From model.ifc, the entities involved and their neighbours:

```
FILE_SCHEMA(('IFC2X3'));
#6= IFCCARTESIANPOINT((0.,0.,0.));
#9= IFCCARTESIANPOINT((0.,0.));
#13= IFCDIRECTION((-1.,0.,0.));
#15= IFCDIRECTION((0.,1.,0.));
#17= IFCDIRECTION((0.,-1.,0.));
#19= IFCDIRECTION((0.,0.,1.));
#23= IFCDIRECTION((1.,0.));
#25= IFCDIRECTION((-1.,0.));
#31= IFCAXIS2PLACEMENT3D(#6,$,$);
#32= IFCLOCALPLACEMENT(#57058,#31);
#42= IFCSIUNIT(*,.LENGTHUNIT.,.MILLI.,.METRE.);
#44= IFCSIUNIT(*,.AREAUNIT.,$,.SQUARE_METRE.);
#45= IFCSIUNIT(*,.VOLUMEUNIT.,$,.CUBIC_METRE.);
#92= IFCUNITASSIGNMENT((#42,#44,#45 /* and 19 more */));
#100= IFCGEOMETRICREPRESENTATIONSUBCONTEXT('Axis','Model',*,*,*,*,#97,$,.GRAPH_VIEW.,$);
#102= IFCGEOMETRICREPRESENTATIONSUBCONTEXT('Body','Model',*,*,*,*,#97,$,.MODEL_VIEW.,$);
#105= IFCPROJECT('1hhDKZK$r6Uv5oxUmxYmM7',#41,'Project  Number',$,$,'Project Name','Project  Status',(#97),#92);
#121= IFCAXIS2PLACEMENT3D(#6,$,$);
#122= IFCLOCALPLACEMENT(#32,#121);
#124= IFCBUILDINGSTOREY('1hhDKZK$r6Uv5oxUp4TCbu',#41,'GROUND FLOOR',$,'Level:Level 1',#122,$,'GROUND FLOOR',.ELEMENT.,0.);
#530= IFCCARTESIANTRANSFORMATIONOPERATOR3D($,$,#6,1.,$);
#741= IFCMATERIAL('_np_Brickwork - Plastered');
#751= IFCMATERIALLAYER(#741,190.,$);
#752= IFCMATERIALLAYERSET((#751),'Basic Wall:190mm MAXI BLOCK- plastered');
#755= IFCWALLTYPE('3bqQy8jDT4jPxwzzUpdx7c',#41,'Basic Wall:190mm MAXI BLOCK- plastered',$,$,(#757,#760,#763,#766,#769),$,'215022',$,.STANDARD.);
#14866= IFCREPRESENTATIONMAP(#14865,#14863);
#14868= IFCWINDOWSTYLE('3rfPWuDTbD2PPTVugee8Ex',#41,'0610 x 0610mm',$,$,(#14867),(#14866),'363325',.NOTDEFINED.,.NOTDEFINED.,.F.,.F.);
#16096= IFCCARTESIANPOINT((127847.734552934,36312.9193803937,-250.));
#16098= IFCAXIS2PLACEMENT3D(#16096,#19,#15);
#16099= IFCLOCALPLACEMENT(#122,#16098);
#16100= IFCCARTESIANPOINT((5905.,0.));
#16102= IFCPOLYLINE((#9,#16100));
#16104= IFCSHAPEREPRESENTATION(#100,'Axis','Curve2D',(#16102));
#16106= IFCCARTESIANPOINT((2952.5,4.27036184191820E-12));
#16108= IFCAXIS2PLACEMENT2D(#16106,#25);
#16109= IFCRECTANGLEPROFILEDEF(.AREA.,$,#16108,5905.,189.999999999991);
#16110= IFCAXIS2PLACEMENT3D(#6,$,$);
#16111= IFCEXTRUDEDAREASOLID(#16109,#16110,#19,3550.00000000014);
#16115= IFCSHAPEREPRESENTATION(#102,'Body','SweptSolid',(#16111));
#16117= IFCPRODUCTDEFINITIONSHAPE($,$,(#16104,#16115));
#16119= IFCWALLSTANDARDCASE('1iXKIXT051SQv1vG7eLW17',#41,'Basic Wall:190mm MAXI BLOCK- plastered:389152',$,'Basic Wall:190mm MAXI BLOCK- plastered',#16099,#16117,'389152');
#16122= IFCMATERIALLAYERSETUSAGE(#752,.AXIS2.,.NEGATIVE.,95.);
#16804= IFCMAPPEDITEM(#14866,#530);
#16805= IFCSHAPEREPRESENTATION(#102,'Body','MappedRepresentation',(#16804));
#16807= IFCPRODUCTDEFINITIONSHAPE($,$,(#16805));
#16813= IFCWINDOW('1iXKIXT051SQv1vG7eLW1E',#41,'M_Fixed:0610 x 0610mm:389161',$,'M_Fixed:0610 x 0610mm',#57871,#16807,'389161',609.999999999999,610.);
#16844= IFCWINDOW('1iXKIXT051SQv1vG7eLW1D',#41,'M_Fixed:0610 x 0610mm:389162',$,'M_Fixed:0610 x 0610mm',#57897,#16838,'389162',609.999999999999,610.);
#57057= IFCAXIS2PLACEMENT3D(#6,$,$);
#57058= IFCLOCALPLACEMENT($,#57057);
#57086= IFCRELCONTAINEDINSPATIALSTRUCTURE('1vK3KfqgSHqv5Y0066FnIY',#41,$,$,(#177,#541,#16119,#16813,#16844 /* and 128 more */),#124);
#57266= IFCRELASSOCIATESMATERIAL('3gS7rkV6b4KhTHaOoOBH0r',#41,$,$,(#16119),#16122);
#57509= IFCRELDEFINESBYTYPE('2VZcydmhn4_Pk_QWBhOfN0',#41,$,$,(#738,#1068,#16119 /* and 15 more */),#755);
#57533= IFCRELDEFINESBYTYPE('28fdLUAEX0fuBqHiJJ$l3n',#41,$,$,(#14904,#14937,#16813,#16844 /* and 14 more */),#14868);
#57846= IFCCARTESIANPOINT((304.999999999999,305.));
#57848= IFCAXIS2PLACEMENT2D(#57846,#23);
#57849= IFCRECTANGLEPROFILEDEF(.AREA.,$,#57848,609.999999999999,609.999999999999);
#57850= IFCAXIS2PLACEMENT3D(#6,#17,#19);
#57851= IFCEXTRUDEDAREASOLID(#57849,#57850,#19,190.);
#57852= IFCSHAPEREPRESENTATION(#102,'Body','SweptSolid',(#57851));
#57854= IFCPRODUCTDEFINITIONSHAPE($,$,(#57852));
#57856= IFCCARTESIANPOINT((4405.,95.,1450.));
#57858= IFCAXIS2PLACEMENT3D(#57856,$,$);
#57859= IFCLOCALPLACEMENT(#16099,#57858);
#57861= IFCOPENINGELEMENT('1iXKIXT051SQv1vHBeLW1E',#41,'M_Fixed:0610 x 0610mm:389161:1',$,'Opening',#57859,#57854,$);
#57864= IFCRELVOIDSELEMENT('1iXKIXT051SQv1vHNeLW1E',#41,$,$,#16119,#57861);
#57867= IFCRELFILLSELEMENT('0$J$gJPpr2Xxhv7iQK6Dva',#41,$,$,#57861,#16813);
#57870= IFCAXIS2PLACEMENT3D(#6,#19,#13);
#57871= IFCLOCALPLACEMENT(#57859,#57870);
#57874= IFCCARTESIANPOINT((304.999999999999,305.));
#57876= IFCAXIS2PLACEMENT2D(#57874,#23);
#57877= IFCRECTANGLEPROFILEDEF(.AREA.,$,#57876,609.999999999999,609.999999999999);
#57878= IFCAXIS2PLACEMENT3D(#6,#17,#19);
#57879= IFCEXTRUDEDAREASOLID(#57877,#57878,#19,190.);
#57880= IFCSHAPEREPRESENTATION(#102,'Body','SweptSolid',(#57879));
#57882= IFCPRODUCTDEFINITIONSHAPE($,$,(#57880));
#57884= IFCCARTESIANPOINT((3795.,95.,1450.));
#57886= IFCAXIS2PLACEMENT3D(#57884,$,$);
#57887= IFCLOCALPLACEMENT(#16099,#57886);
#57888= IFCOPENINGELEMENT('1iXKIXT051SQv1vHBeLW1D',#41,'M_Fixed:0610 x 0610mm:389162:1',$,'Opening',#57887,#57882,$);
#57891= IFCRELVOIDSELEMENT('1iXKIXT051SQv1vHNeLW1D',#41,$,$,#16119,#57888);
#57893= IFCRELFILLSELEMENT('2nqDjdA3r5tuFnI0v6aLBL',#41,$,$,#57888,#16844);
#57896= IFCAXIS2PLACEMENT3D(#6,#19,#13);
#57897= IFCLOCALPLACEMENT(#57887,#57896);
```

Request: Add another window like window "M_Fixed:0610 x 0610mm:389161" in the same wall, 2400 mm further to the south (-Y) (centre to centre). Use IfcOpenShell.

```python
import ifcopenshell
import ifcopenshell.api.feature
import ifcopenshell.api.geometry
import ifcopenshell.api.root
import ifcopenshell.geom
import ifcopenshell.util.element
import ifcopenshell.util.placement
import ifcopenshell.util.shape
import ifcopenshell.util.unit

model = ifcopenshell.open("model.ifc")
unit_scale = ifcopenshell.util.unit.calculate_unit_scale(model)
settings = ifcopenshell.geom.settings()


def volume(element):
    """Net volume in cubic metres, openings subtracted."""
    shape = ifcopenshell.geom.create_shape(settings, element)
    return ifcopenshell.util.shape.get_volume(shape.geometry)


def reuse_history(source, copy):
    """copy_class also copies each property set's owner history, people and application; keep the originals."""
    for rel in copy.IsDefinedBy:
        if rel.is_a("IfcRelDefinesByProperties") and (history := rel.RelatingPropertyDefinition.OwnerHistory):
            rel.RelatingPropertyDefinition.OwnerHistory = source.OwnerHistory
            ifcopenshell.util.element.remove_deep2(model, history)


window = model.by_id(16813)
opening = window.FillsVoids[0].RelatingOpeningElement
wall = opening.VoidsElements[0].RelatingBuildingElement
before = volume(wall)
shift = ifcopenshell.util.placement.get_local_placement(wall.ObjectPlacement)[:3, 0] * -2.4 / unit_scale

# copy_class copies the void relationship, type, container and properties, but no geometry.
new_opening = ifcopenshell.api.root.copy_class(model, product=opening)
new_opening.Representation = ifcopenshell.util.element.copy_deep(
    model, opening.Representation, exclude=["IfcGeometricRepresentationContext", "IfcRepresentationMap"]
)
new_opening.Name = "M_Fixed:0610 x 0610mm"
new_window = ifcopenshell.api.root.copy_class(model, product=window)
new_window.Representation = ifcopenshell.util.element.copy_deep(
    model, window.Representation, exclude=["IfcGeometricRepresentationContext", "IfcRepresentationMap"]
)
new_window.Name = "M_Fixed:0610 x 0610mm"
new_window.Tag = None
reuse_history(window, new_window)
fills = ifcopenshell.api.feature.add_filling(model, opening=new_opening, element=new_window)
fills.OwnerHistory = new_window.OwnerHistory  # required in IFC2X3

for old, new in ((opening, new_opening), (window, new_window)):
    matrix = ifcopenshell.util.placement.get_local_placement(old.ObjectPlacement)
    matrix[:3, 3] += shift
    ifcopenshell.api.geometry.edit_object_placement(model, product=new, matrix=matrix, is_si=False)

after = volume(wall)

print(f"wall volume {before:.3f} -> {after:.3f} m3")

model.write("model_updated.ifc")
```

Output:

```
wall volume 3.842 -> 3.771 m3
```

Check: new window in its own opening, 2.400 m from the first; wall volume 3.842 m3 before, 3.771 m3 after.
